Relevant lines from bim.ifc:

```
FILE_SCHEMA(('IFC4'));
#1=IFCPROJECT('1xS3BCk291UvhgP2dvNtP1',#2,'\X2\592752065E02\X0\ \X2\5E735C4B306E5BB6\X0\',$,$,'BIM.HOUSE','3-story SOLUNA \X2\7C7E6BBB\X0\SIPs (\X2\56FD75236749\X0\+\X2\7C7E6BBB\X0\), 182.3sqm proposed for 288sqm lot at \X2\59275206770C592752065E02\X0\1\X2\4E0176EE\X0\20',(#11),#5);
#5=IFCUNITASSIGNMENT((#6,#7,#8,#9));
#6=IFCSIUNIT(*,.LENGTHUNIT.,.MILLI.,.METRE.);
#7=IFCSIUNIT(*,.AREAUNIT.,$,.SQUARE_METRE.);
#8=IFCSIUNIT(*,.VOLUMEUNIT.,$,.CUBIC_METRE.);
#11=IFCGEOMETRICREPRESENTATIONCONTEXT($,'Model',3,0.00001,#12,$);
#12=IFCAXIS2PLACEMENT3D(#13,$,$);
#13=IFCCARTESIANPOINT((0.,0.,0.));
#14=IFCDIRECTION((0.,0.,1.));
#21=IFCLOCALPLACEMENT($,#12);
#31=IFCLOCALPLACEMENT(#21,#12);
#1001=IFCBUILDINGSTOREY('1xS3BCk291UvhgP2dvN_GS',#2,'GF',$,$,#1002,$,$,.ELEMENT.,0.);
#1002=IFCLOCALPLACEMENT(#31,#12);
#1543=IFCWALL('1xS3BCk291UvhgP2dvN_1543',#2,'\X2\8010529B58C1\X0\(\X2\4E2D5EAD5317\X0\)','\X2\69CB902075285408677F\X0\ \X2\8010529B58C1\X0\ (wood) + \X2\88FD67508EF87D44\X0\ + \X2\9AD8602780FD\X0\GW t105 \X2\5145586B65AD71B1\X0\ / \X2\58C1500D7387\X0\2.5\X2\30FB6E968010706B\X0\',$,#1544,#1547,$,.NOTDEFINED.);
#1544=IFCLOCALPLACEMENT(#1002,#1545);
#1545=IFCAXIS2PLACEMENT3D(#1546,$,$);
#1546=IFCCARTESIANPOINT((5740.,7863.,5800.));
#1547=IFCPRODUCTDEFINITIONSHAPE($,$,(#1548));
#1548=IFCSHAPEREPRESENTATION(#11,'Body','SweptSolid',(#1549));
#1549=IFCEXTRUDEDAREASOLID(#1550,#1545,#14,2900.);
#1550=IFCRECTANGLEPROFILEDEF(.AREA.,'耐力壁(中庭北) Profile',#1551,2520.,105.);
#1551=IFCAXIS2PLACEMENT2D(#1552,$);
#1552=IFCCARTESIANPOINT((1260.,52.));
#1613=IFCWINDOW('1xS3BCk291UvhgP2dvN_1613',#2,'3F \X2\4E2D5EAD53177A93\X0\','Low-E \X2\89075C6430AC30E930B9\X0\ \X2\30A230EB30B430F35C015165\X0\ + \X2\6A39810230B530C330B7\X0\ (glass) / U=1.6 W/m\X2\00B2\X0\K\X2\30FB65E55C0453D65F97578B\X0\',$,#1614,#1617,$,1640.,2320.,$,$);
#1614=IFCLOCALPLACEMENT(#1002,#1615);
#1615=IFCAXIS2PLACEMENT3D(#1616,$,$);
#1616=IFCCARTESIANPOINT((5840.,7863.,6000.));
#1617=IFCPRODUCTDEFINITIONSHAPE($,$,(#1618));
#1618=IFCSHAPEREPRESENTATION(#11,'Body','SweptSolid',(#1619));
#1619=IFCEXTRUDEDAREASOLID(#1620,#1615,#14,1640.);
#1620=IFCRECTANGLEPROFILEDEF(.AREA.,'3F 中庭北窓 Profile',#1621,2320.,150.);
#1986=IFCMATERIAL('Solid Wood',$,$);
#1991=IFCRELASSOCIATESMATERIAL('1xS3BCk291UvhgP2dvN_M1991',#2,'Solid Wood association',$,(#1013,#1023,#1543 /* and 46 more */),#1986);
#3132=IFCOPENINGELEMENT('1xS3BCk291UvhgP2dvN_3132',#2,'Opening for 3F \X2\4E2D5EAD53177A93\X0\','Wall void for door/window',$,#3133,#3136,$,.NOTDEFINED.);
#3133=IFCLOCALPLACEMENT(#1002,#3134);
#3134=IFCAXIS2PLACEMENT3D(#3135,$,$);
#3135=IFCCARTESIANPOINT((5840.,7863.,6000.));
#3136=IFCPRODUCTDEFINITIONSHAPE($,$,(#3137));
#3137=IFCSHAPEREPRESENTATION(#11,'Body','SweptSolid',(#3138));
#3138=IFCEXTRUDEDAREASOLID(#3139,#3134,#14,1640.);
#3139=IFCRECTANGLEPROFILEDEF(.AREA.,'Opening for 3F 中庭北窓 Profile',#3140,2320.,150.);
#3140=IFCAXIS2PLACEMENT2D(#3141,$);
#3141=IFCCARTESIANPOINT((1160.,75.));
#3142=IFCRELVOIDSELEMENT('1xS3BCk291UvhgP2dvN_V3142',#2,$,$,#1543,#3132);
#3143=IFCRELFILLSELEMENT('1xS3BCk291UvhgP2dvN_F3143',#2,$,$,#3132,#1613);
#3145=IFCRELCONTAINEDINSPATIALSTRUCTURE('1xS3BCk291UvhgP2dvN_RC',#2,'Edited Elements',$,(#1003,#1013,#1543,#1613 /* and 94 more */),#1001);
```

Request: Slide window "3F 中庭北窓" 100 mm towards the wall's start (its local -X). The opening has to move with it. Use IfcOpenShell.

```python
import ifcopenshell
import ifcopenshell.api.geometry
import ifcopenshell.util.placement

model = ifcopenshell.open("bim.ifc")

window = model.by_guid("1xS3BCk291UvhgP2dvN_1613")
opening = window.FillsVoids[0].RelatingOpeningElement
wall = opening.VoidsElements[0].RelatingBuildingElement

wall_matrix = ifcopenshell.util.placement.get_local_placement(wall.ObjectPlacement)
shift = wall_matrix[:3, 0] * -100.0
before = ifcopenshell.util.placement.get_local_placement(window.ObjectPlacement)[:3, 3].copy()

# The window is not placed relative to its opening, so move both.
for product in (opening, window):
    matrix = ifcopenshell.util.placement.get_local_placement(product.ObjectPlacement)
    matrix[:3, 3] += shift
    ifcopenshell.api.geometry.edit_object_placement(model, product=product, matrix=matrix, is_si=False)

after = ifcopenshell.util.placement.get_local_placement(window.ObjectPlacement)[:3, 3]
print("window moved by", (after - before).round(3) + 0.0)

model.write("bim_updated.ifc")
```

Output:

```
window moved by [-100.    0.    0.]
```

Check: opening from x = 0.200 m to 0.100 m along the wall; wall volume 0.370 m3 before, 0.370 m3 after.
